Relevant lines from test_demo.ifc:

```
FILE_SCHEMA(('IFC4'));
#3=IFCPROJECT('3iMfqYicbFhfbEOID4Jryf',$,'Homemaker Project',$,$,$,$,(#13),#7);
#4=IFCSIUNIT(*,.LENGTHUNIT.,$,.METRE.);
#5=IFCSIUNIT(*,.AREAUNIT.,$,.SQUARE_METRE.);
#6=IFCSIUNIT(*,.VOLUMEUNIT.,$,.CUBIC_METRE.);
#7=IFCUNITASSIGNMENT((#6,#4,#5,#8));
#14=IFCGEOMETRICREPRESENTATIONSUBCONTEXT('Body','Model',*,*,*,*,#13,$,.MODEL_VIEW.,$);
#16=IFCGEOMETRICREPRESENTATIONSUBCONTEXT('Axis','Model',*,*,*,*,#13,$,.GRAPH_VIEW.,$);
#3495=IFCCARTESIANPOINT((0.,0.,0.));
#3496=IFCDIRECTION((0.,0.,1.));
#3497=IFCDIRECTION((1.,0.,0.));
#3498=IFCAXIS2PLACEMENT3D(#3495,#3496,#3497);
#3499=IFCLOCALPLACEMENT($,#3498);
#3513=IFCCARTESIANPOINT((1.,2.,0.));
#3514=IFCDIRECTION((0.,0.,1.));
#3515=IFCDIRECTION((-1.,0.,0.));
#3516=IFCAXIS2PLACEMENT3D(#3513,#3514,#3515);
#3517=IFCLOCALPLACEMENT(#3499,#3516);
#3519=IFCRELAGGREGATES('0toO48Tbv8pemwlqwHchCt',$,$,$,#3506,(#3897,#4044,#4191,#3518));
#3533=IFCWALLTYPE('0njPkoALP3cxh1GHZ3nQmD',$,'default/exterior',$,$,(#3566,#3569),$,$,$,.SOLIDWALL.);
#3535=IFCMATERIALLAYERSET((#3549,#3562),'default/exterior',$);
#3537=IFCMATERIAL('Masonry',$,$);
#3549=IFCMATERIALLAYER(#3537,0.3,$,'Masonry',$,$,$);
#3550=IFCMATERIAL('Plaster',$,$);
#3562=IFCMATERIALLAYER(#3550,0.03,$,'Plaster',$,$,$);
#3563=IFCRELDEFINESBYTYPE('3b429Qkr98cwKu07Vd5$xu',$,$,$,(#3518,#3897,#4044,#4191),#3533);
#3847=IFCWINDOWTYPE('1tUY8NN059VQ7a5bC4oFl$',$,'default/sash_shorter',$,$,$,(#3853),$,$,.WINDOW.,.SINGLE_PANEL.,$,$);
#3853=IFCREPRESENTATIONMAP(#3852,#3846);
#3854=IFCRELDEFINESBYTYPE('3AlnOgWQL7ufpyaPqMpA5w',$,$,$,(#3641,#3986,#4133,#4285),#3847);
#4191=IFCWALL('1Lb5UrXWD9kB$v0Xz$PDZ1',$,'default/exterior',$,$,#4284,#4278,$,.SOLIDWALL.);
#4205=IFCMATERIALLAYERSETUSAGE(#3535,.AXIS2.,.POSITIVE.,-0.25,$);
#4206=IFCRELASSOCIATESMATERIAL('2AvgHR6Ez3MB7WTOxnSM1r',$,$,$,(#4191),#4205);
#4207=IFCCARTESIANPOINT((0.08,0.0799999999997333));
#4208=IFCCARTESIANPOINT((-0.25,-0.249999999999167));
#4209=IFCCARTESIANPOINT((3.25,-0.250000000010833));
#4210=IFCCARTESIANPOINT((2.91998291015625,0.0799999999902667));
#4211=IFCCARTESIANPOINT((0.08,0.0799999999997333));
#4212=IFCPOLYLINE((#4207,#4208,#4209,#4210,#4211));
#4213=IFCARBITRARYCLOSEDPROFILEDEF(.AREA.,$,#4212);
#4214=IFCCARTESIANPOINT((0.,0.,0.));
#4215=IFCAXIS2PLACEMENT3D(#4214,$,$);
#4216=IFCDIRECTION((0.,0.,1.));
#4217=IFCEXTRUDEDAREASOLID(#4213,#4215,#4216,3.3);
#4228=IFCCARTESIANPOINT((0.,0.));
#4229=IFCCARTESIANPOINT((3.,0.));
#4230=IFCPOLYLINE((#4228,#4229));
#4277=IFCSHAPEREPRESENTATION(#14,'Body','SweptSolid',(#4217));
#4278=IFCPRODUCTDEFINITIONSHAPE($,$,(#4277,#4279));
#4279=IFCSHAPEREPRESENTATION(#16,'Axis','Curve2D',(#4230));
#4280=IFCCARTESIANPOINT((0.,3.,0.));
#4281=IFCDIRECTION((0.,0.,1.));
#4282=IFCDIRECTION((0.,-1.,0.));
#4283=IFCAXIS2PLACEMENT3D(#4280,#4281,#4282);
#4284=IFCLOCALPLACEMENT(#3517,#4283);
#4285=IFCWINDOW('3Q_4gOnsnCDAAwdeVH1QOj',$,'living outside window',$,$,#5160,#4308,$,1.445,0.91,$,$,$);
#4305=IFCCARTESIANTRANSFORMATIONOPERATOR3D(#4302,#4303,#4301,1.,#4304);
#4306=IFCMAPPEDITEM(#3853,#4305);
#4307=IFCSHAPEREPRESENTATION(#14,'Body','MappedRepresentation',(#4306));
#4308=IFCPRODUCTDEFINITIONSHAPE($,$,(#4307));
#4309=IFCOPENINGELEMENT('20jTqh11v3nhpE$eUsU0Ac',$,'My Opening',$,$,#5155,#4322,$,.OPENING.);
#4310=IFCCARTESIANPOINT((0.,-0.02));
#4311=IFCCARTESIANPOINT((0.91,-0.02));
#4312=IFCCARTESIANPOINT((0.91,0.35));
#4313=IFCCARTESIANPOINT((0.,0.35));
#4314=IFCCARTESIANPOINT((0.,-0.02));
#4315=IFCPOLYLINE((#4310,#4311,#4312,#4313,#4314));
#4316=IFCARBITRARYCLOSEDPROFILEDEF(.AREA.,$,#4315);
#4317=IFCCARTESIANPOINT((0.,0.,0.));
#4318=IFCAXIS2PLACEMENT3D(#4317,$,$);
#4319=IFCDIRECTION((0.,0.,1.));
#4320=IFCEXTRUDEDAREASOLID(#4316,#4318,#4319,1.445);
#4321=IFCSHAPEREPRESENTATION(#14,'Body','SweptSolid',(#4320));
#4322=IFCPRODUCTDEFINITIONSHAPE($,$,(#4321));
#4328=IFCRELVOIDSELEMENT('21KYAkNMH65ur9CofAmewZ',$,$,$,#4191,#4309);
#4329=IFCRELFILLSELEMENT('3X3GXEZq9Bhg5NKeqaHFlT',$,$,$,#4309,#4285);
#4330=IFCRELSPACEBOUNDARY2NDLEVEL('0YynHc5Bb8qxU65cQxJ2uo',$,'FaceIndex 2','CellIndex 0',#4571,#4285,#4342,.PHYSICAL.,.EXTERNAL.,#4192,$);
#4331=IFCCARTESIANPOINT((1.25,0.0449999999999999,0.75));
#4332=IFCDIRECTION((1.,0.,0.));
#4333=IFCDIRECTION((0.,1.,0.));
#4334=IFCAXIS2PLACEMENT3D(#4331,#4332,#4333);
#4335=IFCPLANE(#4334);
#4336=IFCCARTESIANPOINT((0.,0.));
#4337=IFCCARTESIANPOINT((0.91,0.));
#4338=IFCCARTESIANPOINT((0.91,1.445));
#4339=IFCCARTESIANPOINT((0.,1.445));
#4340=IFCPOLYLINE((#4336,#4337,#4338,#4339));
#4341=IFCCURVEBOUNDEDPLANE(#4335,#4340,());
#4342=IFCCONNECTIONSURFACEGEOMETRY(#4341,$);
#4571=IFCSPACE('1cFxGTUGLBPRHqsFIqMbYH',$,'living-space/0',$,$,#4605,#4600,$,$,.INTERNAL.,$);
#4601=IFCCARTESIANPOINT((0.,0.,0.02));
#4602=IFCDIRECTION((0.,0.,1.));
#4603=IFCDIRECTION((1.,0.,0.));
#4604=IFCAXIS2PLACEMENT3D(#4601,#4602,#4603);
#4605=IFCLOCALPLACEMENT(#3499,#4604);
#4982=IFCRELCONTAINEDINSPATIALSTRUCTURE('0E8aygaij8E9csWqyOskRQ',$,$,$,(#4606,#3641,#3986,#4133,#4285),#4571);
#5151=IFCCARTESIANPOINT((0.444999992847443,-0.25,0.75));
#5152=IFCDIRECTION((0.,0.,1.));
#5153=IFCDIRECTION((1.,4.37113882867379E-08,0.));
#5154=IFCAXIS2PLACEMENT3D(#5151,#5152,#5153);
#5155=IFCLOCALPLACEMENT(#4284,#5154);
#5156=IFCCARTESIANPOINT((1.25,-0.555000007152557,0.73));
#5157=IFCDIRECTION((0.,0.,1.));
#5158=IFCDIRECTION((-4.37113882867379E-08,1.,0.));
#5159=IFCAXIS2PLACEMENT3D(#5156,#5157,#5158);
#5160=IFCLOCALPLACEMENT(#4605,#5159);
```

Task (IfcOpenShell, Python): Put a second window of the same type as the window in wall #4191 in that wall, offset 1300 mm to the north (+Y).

```python
import numpy as np
import ifcopenshell
import ifcopenshell.api.feature
import ifcopenshell.api.geometry
import ifcopenshell.api.root
import ifcopenshell.geom
import ifcopenshell.util.element
import ifcopenshell.util.placement
import ifcopenshell.util.shape

model = ifcopenshell.open("test_demo.ifc")
settings = ifcopenshell.geom.settings()


def volume(element):
    """Net volume in cubic metres, openings subtracted."""
    shape = ifcopenshell.geom.create_shape(settings, element)
    return ifcopenshell.util.shape.get_volume(shape.geometry)


window = model.by_id(4285)
opening = window.FillsVoids[0].RelatingOpeningElement
wall = opening.VoidsElements[0].RelatingBuildingElement
before = volume(wall)
shift = ifcopenshell.util.placement.get_local_placement(wall.ObjectPlacement)[:3, 0] * 1.3

# copy_class copies the void relationship, type, container and properties, but no geometry.
new_opening = ifcopenshell.api.root.copy_class(model, product=opening)
new_opening.Representation = ifcopenshell.util.element.copy_deep(
    model, opening.Representation, exclude=["IfcGeometricRepresentationContext", "IfcRepresentationMap"]
)
new_window = ifcopenshell.api.root.copy_class(model, product=window)
new_window.Representation = ifcopenshell.util.element.copy_deep(
    model, window.Representation, exclude=["IfcGeometricRepresentationContext", "IfcRepresentationMap"]
)
ifcopenshell.api.feature.add_filling(model, opening=new_opening, element=new_window)

for old, new in ((opening, new_opening), (window, new_window)):
    matrix = ifcopenshell.util.placement.get_local_placement(old.ObjectPlacement)
    matrix[:3, 3] += shift
    ifcopenshell.api.geometry.edit_object_placement(model, product=new, matrix=matrix, is_si=False)

# The copied space boundaries still share their surfaces with the original.
for rel in new_window.ProvidesBoundaries:
    if rel.ConnectionGeometry:
        rel.ConnectionGeometry = ifcopenshell.util.element.copy_deep(model, rel.ConnectionGeometry)

# Space boundary surfaces are stored in each space's coordinates; move them too.
for rel in new_window.ProvidesBoundaries:
    if not rel.ConnectionGeometry:
        continue
    surface = rel.ConnectionGeometry.SurfaceOnRelatingElement.BasisSurface
    space_matrix = ifcopenshell.util.placement.get_local_placement(rel.RelatingSpace.ObjectPlacement)
    point = np.array(surface.Position.Location.Coordinates) + space_matrix[:3, :3].T @ shift
    surface.Position = model.createIfcAxis2Placement3D(
        model.createIfcCartesianPoint(point.tolist()), surface.Position.Axis, surface.Position.RefDirection
    )

after = volume(wall)

print(f"wall volume {before:.3f} -> {after:.3f} m3")

model.write("test_demo_v2.ifc")
```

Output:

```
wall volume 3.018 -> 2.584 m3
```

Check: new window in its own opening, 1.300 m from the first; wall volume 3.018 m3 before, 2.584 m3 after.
